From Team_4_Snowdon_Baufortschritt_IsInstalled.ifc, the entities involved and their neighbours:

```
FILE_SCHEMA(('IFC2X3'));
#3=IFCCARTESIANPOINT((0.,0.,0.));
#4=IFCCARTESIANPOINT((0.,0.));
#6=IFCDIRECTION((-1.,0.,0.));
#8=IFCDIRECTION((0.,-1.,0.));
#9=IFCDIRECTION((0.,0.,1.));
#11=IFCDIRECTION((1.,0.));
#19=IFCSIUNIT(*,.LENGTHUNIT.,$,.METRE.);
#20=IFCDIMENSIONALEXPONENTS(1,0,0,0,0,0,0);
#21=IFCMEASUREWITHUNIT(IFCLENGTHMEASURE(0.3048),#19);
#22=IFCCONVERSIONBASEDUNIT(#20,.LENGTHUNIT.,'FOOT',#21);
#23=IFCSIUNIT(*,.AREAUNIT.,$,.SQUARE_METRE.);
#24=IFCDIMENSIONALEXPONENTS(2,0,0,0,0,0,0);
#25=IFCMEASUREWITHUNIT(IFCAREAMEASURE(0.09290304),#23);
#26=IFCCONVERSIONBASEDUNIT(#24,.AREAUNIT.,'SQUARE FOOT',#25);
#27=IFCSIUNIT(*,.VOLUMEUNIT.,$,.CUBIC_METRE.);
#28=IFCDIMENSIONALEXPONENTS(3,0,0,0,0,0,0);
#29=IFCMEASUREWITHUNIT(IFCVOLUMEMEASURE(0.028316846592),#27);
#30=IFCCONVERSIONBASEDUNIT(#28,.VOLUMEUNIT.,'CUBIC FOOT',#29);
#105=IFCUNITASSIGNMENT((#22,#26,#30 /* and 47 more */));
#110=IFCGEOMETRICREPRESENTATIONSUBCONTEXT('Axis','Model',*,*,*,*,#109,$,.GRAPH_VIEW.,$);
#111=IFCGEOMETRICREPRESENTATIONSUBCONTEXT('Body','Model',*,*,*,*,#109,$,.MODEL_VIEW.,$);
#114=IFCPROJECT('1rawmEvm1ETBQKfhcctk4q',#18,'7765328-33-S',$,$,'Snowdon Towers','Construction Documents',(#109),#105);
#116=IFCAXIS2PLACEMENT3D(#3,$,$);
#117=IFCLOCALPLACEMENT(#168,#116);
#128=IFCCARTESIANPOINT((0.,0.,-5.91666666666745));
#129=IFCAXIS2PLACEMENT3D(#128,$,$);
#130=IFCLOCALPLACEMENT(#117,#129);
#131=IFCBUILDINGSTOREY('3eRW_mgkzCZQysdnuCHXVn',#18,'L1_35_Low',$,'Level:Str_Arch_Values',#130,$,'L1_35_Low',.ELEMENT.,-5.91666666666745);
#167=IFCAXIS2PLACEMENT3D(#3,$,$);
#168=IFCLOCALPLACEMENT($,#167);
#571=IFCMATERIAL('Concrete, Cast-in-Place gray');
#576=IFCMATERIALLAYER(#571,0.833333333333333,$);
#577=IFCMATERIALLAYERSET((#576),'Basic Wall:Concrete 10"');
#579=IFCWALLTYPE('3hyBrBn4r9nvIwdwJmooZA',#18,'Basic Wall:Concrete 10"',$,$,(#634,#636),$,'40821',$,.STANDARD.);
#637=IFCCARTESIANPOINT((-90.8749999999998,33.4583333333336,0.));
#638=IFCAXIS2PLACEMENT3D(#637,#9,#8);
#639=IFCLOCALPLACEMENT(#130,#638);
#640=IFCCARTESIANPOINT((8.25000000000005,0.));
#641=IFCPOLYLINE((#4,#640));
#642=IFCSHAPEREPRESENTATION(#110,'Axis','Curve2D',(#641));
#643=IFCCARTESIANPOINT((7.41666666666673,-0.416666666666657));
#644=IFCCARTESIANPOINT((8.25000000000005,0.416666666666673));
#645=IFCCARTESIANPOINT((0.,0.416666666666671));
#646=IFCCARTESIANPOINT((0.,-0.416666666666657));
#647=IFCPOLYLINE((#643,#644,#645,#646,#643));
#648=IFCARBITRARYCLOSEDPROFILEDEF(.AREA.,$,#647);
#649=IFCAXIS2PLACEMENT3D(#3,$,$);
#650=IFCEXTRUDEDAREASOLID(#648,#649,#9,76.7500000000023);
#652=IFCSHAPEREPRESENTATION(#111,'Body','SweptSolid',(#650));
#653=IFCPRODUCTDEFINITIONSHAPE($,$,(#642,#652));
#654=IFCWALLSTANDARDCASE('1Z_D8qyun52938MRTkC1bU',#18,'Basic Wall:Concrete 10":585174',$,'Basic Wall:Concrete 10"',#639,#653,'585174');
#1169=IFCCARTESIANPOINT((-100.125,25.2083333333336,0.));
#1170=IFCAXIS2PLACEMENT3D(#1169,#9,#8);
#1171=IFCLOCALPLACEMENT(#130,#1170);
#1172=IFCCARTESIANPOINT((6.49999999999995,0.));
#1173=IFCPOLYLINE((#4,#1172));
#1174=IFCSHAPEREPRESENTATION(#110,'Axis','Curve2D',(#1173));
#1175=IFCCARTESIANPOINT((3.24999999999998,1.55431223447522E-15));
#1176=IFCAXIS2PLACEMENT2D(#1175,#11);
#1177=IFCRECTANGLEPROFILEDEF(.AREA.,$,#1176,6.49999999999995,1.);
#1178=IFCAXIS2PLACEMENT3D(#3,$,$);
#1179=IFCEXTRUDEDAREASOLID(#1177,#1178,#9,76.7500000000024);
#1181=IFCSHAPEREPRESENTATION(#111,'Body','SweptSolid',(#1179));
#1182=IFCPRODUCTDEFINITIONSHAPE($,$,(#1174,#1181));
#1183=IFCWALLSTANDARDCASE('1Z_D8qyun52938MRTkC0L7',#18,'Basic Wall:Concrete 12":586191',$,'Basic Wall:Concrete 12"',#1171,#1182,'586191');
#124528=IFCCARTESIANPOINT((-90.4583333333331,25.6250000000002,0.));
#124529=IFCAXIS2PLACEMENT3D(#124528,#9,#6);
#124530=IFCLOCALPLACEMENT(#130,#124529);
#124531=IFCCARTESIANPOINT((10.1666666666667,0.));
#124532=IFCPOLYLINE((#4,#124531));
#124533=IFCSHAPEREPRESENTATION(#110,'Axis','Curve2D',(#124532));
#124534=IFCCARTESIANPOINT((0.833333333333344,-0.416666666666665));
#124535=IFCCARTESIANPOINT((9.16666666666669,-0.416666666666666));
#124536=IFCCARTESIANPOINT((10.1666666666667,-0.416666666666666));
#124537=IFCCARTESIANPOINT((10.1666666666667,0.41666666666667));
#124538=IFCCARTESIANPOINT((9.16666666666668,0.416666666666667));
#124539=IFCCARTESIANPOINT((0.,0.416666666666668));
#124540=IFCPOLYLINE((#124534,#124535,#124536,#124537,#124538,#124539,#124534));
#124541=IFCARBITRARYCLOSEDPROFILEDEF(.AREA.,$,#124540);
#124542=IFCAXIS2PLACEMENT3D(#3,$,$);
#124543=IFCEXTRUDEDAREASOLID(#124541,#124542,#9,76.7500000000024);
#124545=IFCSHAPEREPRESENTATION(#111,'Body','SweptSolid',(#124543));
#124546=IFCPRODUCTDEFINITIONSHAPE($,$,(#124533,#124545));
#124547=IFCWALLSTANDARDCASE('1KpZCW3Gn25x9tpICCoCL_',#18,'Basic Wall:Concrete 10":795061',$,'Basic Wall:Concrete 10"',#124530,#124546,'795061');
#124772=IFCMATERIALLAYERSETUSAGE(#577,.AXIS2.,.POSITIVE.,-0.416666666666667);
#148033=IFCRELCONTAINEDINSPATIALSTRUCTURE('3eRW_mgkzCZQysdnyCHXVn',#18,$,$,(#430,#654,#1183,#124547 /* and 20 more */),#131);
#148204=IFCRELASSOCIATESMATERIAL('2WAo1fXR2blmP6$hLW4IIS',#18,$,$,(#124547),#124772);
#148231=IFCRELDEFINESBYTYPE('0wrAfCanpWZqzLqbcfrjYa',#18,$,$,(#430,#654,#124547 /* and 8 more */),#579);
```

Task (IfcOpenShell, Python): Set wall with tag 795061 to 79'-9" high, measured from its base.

```python
import ifcopenshell
import ifcopenshell.geom
import ifcopenshell.util.representation
import ifcopenshell.util.shape
import ifcopenshell.util.unit

model = ifcopenshell.open("Team_4_Snowdon_Baufortschritt_IsInstalled.ifc")
unit_scale = ifcopenshell.util.unit.calculate_unit_scale(model)
settings = ifcopenshell.geom.settings()


def volume(element):
    """Net volume in cubic metres, openings subtracted."""
    shape = ifcopenshell.geom.create_shape(settings, element)
    return ifcopenshell.util.shape.get_volume(shape.geometry)


wall = model.by_id(124547)
before = volume(wall)

body = ifcopenshell.util.representation.get_representation(wall, "Model", "Body")
solid = body.Items[0]
old_height = solid.Depth
solid.Depth = 957 * 0.0254 / unit_scale
after = volume(wall)

print(f"height {old_height:g} -> {solid.Depth:g}, volume {before:.3f} -> {after:.3f} m3")

model.write("Team_4_Snowdon_Baufortschritt_IsInstalled-out.ifc")
```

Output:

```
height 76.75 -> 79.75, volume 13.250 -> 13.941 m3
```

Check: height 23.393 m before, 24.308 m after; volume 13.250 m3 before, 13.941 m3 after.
